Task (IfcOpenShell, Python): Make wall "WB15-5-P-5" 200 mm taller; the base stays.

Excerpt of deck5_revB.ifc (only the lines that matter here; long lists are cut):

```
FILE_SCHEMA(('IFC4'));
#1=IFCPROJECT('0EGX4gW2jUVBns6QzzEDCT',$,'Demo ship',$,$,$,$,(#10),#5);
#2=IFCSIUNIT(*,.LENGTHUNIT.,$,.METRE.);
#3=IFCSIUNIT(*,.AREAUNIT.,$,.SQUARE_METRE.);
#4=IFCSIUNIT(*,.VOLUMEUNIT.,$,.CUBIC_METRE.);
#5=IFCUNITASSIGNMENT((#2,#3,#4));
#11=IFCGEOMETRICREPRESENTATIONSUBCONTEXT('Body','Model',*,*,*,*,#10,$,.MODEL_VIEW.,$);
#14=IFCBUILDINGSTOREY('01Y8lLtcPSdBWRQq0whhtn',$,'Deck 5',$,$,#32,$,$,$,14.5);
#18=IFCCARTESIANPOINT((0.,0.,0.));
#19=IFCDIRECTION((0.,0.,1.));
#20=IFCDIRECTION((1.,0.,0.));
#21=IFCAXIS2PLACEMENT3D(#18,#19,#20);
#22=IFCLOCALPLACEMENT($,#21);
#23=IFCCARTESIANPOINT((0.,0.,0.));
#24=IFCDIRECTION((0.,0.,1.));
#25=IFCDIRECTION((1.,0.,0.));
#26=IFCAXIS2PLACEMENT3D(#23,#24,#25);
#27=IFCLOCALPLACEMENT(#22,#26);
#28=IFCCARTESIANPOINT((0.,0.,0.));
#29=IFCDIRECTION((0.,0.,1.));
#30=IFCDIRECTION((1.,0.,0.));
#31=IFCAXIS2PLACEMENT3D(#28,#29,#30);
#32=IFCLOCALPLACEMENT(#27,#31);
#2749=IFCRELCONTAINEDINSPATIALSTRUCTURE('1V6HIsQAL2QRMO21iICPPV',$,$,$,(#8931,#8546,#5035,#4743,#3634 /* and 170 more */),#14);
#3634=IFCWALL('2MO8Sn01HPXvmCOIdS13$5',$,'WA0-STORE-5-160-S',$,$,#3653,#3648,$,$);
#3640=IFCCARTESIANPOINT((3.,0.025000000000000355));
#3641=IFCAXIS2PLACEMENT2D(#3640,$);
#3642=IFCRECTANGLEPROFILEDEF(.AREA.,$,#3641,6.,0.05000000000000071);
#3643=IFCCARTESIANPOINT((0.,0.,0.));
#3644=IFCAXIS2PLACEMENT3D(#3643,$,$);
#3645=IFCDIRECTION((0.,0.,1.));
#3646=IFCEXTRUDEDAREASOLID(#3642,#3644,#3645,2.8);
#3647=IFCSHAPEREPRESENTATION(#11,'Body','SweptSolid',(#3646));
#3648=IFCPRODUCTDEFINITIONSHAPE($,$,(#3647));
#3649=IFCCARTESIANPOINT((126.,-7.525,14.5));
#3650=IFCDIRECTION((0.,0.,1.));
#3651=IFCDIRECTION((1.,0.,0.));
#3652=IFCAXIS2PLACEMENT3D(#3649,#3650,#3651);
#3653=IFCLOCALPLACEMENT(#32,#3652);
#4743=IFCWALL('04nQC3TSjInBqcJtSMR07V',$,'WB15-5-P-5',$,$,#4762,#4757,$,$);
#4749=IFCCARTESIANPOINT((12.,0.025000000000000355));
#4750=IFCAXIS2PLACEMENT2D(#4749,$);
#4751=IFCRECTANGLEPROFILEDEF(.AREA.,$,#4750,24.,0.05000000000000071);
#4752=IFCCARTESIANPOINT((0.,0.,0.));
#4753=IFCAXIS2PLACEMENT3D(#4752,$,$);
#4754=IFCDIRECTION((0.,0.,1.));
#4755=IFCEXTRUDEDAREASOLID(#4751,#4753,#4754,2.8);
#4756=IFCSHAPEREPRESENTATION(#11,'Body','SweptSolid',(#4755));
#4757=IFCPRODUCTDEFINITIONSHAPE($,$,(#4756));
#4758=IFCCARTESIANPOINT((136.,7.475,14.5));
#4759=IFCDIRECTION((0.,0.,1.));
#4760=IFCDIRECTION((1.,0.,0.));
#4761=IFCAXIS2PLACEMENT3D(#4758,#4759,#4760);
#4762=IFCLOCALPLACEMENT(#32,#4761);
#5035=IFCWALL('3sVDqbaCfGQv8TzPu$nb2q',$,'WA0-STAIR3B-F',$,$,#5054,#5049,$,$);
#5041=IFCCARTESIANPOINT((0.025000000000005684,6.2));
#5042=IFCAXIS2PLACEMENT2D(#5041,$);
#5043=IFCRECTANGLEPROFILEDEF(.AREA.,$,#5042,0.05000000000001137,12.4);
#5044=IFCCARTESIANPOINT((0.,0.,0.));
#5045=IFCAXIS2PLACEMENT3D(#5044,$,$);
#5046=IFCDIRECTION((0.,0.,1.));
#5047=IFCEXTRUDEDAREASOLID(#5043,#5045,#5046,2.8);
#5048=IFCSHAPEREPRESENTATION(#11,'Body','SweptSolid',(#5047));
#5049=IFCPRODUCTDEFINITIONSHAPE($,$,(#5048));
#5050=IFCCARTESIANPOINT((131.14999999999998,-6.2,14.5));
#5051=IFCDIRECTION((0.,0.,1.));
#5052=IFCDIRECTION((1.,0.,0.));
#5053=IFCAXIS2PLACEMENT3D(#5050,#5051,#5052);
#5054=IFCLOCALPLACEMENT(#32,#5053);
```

```python
import ifcopenshell
import ifcopenshell.geom
import ifcopenshell.util.representation
import ifcopenshell.util.shape
import ifcopenshell.util.unit

model = ifcopenshell.open("deck5_revB.ifc")
unit_scale = ifcopenshell.util.unit.calculate_unit_scale(model)
settings = ifcopenshell.geom.settings()


def volume(element):
    """Net volume in cubic metres, openings subtracted."""
    shape = ifcopenshell.geom.create_shape(settings, element)
    return ifcopenshell.util.shape.get_volume(shape.geometry)


wall = model.by_guid("04nQC3TSjInBqcJtSMR07V")
before = volume(wall)

body = ifcopenshell.util.representation.get_representation(wall, "Model", "Body")
solid = body.Items[0]
old_height = solid.Depth
solid.Depth += 0.2 / unit_scale
after = volume(wall)

print(f"height {old_height:g} -> {solid.Depth:g}, volume {before:.3f} -> {after:.3f} m3")

model.write("deck5_revB_v2.ifc")
```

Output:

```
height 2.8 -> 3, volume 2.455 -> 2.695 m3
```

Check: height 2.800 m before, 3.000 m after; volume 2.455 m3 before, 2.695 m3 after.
